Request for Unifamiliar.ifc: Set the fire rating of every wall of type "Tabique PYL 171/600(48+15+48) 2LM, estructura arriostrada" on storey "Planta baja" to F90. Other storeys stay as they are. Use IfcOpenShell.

First a look at what the model holds.

```python
import ifcopenshell
import ifcopenshell.util.element

model = ifcopenshell.open("Unifamiliar.ifc")
print(model.schema)
storey = next(s for s in model.by_type("IfcBuildingStorey") if s.Name == "Planta baja")
walls = [e for e in ifcopenshell.util.element.get_decomposition(storey) if e.is_a("IfcWall")]
seen = {}
for e in walls:
    element_type = ifcopenshell.util.element.get_type(e)
    key = (element_type.Name if element_type != e and element_type else None, ifcopenshell.util.element.get_pset(e, "Pset_WallCommon", "FireRating"))
    seen[key] = seen.get(key, 0) + 1
for (name, value), count in sorted(seen.items(), key=str):
    print(count, "x", name, "|", value)
```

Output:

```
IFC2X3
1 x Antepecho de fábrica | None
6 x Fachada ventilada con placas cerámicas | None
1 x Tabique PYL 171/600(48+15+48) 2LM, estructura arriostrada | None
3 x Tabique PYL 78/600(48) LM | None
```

```python
import ifcopenshell
import ifcopenshell.api.pset
import ifcopenshell.util.element

model = ifcopenshell.open("Unifamiliar.ifc")

storey = next(s for s in model.by_type("IfcBuildingStorey") if s.Name == "Planta baja")
walls = [e for e in ifcopenshell.util.element.get_decomposition(storey) if e.is_a("IfcWall")]

count = 0
for e in walls:
    element_type = ifcopenshell.util.element.get_type(e)
    if element_type in (None, e) or element_type.Name != "Tabique PYL 171/600(48+15+48) 2LM, estructura arriostrada":
        continue
    # add_pset returns the element's existing set when there is one.
    pset = ifcopenshell.api.pset.add_pset(model, product=e, name="Pset_WallCommon")
    ifcopenshell.api.pset.edit_pset(model, pset=pset, properties={"FireRating": "F90"})
    count += 1

print(count, "walls updated")

model.write("Unifamiliar_edited.ifc")
```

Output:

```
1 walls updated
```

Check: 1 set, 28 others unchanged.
